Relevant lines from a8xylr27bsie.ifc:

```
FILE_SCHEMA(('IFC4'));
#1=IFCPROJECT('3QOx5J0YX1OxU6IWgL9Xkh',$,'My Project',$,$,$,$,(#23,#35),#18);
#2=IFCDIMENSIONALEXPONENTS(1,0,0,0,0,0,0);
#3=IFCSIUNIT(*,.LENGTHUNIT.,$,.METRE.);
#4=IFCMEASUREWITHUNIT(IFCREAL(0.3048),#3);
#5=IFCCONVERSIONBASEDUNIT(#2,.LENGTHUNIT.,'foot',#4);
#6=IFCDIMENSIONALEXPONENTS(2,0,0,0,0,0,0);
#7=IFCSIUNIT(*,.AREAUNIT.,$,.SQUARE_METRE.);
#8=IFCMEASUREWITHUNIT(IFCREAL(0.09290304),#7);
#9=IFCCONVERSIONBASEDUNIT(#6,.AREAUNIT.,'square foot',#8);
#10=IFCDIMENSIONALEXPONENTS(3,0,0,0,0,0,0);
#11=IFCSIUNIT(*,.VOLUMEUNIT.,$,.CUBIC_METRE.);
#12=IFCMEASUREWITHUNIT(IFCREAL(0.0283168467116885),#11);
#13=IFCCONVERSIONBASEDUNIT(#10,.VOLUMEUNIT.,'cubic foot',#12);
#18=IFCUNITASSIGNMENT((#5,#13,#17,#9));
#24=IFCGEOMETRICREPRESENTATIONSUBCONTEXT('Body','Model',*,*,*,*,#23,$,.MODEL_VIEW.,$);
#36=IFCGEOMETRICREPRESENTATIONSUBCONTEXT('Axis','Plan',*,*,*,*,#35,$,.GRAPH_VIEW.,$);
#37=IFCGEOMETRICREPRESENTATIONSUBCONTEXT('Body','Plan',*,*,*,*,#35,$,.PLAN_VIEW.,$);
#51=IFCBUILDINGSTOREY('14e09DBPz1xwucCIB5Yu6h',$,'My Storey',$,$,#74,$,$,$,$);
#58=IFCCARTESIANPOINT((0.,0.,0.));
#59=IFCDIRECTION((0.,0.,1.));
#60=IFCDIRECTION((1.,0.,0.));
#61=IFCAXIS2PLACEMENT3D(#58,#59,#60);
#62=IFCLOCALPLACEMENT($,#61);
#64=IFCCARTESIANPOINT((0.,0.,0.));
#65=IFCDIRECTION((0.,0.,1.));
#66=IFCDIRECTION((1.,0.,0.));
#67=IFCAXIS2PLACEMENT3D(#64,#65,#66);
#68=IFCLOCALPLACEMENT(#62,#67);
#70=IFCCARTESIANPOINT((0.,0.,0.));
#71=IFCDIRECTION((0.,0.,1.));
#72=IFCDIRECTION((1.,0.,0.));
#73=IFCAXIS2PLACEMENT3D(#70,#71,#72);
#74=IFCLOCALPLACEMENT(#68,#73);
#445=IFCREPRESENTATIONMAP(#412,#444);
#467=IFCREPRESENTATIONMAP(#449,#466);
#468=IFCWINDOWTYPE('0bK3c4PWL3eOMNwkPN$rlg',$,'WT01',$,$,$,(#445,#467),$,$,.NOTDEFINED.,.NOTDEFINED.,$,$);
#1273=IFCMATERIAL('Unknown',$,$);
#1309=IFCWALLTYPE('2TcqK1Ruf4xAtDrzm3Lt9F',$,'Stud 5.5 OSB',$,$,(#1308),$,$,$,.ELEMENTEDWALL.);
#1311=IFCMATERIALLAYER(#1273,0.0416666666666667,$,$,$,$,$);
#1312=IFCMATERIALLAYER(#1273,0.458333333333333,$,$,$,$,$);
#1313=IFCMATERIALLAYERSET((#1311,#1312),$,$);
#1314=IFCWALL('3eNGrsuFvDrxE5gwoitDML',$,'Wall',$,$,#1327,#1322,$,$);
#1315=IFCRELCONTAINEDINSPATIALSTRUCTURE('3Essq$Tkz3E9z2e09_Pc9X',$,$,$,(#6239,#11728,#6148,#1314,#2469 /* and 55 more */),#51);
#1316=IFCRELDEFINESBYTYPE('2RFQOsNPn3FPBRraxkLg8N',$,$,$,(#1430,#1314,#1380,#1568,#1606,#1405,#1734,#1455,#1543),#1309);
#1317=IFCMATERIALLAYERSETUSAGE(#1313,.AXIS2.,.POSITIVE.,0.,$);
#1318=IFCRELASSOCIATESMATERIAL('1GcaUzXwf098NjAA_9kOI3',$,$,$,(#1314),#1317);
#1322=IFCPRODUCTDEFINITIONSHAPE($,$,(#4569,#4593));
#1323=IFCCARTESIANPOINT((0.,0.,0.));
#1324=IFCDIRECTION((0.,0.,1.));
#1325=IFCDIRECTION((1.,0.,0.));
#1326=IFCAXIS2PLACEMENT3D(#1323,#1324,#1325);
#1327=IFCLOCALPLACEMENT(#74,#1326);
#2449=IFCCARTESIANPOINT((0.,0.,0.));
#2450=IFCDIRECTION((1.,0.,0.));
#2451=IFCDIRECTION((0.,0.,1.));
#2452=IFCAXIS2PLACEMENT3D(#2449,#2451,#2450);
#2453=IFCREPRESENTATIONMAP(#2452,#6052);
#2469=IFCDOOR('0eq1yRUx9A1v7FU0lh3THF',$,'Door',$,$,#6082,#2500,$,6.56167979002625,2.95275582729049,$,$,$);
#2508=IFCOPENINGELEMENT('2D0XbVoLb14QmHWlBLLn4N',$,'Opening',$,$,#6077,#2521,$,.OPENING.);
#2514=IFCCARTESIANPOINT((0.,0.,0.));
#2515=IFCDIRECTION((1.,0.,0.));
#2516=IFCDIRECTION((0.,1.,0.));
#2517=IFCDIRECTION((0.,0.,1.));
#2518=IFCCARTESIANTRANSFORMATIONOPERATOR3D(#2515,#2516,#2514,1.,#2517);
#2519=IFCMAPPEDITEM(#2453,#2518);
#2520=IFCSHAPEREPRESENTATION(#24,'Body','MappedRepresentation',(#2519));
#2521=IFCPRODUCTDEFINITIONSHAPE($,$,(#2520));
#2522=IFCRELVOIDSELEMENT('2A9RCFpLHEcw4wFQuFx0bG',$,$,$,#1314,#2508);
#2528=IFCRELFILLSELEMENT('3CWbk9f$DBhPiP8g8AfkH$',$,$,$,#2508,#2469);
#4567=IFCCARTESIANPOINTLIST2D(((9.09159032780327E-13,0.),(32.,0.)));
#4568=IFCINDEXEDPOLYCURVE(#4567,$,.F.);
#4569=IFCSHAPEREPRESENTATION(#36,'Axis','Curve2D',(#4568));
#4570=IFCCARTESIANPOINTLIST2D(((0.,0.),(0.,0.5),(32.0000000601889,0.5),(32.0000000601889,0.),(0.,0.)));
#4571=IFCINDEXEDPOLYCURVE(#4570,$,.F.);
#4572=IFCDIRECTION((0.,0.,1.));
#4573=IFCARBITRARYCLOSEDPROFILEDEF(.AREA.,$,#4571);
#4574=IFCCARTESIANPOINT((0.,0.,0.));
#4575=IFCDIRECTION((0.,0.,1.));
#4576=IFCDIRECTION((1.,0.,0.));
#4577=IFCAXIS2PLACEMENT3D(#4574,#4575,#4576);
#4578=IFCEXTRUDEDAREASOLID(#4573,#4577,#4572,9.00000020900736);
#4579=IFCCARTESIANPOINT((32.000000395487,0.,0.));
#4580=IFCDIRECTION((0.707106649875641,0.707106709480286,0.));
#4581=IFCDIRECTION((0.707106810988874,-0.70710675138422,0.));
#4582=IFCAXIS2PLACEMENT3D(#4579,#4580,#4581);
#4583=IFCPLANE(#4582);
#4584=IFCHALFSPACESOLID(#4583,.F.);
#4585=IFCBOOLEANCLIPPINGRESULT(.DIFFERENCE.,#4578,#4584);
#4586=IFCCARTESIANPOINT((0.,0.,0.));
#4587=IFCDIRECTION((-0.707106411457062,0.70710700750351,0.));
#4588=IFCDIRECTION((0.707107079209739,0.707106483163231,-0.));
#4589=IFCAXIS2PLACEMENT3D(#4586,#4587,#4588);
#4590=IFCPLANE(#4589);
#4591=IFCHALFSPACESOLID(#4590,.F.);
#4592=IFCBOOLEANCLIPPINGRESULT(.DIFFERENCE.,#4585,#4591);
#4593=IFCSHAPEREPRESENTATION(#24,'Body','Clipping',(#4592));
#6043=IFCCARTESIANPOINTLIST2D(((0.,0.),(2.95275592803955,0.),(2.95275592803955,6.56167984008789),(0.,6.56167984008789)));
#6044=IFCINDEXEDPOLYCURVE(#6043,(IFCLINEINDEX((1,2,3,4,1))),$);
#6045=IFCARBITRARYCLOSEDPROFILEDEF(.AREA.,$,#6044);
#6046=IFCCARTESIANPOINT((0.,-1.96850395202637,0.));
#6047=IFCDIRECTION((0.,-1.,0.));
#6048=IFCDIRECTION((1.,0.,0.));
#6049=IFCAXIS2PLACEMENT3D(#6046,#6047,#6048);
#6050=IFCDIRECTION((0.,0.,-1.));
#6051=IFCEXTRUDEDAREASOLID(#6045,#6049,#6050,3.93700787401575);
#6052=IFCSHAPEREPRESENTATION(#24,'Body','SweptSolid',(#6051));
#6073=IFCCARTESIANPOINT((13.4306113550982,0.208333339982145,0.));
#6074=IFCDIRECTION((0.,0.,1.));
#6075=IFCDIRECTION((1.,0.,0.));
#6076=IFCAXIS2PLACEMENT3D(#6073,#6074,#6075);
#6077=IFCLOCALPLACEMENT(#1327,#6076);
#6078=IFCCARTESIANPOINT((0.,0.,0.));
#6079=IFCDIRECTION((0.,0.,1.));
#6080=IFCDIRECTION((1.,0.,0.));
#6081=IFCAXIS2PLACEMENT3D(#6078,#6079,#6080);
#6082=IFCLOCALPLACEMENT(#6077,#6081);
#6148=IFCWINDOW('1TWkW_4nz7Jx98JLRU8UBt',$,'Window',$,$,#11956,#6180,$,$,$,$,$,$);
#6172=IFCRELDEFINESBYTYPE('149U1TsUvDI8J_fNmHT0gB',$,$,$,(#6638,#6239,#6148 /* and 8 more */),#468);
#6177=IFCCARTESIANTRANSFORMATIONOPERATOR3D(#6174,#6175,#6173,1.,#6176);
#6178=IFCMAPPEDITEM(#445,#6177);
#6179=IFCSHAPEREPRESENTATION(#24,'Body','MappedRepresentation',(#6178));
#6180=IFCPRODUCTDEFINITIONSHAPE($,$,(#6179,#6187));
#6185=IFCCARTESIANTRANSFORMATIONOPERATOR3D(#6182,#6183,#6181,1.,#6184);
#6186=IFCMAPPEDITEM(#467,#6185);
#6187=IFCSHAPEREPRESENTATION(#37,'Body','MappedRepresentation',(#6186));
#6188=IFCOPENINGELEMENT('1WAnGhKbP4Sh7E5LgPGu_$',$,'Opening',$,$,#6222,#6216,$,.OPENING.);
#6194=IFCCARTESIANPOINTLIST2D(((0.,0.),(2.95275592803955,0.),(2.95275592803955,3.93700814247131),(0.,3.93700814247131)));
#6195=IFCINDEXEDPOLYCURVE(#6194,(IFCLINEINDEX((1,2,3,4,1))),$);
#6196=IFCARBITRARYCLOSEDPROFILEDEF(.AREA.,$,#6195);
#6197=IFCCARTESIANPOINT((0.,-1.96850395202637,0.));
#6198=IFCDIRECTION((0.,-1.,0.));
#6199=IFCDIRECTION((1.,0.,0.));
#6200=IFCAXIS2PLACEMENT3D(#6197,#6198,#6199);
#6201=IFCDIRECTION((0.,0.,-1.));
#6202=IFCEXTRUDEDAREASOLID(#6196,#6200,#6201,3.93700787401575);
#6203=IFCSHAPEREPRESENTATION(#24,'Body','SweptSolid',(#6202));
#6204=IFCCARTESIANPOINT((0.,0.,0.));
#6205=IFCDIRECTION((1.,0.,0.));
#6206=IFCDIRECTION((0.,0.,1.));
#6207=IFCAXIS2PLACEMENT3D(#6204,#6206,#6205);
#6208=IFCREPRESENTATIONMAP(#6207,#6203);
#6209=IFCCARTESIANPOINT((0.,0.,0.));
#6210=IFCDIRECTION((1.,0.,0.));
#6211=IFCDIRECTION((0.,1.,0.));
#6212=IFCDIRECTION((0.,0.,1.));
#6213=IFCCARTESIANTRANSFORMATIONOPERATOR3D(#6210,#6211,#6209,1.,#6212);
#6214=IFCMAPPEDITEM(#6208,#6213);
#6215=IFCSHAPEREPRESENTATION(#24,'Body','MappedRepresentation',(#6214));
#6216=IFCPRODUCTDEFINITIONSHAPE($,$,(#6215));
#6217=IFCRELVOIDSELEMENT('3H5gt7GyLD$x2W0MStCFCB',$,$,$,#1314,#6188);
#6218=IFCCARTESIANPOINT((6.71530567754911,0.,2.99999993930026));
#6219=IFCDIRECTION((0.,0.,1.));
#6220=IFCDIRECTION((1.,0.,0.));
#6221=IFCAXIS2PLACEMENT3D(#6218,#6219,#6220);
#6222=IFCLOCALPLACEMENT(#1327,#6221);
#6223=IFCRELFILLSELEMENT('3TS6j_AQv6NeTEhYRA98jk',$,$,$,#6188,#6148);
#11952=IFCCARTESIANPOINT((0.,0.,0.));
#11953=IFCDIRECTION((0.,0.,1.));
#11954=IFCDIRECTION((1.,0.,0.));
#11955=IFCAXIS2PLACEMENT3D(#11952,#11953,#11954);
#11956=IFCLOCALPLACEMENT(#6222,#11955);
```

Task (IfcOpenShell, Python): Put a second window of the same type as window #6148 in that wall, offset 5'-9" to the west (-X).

```python
import ifcopenshell
import ifcopenshell.api.feature
import ifcopenshell.api.geometry
import ifcopenshell.api.root
import ifcopenshell.geom
import ifcopenshell.util.element
import ifcopenshell.util.placement
import ifcopenshell.util.shape
import ifcopenshell.util.unit

model = ifcopenshell.open("a8xylr27bsie.ifc")
unit_scale = ifcopenshell.util.unit.calculate_unit_scale(model)
settings = ifcopenshell.geom.settings()


def volume(element):
    """Net volume in cubic metres, openings subtracted."""
    shape = ifcopenshell.geom.create_shape(settings, element)
    return ifcopenshell.util.shape.get_volume(shape.geometry)


window = model.by_guid("1TWkW_4nz7Jx98JLRU8UBt")
opening = window.FillsVoids[0].RelatingOpeningElement
wall = opening.VoidsElements[0].RelatingBuildingElement
before = volume(wall)
shift = ifcopenshell.util.placement.get_local_placement(wall.ObjectPlacement)[:3, 0] * -69 * 0.0254 / unit_scale

# copy_class copies the void relationship, type, container and properties, but no geometry.
new_opening = ifcopenshell.api.root.copy_class(model, product=opening)
new_opening.Representation = ifcopenshell.util.element.copy_deep(
    model, opening.Representation, exclude=["IfcGeometricRepresentationContext", "IfcRepresentationMap"]
)
new_window = ifcopenshell.api.root.copy_class(model, product=window)
new_window.Representation = ifcopenshell.util.element.copy_deep(
    model, window.Representation, exclude=["IfcGeometricRepresentationContext", "IfcRepresentationMap"]
)
ifcopenshell.api.feature.add_filling(model, opening=new_opening, element=new_window)

for old, new in ((opening, new_opening), (window, new_window)):
    matrix = ifcopenshell.util.placement.get_local_placement(old.ObjectPlacement)
    matrix[:3, 3] += shift
    ifcopenshell.api.geometry.edit_object_placement(model, product=new, matrix=matrix, is_si=False)

after = volume(wall)

print(f"wall volume {before:.3f} -> {after:.3f} m3")

model.write("a8xylr27bsie_updated.ifc")
```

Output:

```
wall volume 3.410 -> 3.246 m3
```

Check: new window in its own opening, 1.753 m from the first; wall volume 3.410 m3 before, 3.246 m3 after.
